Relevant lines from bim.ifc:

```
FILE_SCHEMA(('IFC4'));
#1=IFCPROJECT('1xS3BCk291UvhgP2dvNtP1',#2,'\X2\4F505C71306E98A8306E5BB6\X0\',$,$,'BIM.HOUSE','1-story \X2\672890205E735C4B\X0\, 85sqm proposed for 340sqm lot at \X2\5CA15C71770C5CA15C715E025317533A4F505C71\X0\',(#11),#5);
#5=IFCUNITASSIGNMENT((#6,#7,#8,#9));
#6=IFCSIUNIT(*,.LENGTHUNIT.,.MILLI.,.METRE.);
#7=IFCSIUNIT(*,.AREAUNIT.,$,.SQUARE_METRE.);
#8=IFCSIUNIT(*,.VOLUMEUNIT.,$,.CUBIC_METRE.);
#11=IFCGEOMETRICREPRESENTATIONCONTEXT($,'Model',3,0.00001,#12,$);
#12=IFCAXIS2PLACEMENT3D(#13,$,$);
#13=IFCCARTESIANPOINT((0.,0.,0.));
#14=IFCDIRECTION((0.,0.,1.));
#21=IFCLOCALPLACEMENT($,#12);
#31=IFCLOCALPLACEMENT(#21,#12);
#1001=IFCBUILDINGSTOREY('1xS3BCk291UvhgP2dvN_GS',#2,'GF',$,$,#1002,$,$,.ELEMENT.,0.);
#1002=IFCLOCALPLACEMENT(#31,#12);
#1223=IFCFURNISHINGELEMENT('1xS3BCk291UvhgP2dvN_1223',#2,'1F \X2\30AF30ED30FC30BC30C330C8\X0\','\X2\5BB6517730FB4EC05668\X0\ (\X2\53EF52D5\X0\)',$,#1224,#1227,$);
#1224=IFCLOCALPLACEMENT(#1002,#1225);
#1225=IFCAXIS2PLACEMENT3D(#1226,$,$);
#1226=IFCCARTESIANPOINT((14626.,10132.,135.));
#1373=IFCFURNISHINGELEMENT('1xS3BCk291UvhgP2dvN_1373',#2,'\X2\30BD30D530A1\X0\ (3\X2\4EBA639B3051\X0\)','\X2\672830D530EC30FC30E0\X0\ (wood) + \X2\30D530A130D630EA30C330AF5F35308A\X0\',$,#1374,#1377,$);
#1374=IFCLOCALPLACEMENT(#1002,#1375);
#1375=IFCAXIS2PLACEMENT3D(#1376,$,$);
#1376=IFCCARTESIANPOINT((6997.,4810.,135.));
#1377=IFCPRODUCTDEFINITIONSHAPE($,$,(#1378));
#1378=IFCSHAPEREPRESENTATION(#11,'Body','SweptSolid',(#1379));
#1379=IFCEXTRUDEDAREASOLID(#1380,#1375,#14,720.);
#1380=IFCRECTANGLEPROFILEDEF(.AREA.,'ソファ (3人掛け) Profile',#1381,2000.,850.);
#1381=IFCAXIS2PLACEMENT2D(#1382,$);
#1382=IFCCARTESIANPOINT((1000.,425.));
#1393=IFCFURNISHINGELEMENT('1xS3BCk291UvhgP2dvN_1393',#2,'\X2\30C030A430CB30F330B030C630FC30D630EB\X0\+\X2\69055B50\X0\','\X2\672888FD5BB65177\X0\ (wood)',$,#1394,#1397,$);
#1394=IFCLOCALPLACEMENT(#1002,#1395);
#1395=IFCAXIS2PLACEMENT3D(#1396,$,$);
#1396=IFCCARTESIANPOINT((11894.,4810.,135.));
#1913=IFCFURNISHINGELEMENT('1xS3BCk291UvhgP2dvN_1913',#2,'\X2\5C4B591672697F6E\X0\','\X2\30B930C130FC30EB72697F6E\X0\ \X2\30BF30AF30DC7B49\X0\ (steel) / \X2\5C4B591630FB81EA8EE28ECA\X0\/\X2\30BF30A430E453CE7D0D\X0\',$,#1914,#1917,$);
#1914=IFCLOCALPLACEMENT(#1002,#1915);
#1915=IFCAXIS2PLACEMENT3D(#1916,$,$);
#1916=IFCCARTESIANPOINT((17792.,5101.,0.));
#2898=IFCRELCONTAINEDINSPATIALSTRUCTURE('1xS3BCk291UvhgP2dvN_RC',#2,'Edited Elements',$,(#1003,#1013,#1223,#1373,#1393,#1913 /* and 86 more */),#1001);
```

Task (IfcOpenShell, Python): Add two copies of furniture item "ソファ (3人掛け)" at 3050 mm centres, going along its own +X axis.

```python
import ifcopenshell
import ifcopenshell.api.geometry
import ifcopenshell.api.root
import ifcopenshell.util.element
import ifcopenshell.util.placement

model = ifcopenshell.open("bim.ifc")


def reuse_history(source, copy):
    """copy_class also copies each property set's owner history, people and application; keep the originals."""
    for rel in copy.IsDefinedBy:
        if rel.is_a("IfcRelDefinesByProperties") and (history := rel.RelatingPropertyDefinition.OwnerHistory):
            rel.RelatingPropertyDefinition.OwnerHistory = source.OwnerHistory
            ifcopenshell.util.element.remove_deep2(model, history)


source = model.by_id(1373)
base = ifcopenshell.util.placement.get_local_placement(source.ObjectPlacement)
step = base[:3, 0] * 3050.0

for i in range(1, 3):
    copy = ifcopenshell.api.root.copy_class(model, product=source)
    copy.Representation = ifcopenshell.util.element.copy_deep(
        model, source.Representation, exclude=["IfcGeometricRepresentationContext", "IfcRepresentationMap"]
    )
    reuse_history(source, copy)
    matrix = base.copy()
    matrix[:3, 3] += i * step
    print("added at", matrix[:3, 3].round(3) + 0.0)
    ifcopenshell.api.geometry.edit_object_placement(model, product=copy, matrix=matrix, is_si=False)

model.write("bim-out.ifc")
```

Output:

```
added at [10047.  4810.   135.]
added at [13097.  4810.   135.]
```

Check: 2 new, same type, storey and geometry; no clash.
